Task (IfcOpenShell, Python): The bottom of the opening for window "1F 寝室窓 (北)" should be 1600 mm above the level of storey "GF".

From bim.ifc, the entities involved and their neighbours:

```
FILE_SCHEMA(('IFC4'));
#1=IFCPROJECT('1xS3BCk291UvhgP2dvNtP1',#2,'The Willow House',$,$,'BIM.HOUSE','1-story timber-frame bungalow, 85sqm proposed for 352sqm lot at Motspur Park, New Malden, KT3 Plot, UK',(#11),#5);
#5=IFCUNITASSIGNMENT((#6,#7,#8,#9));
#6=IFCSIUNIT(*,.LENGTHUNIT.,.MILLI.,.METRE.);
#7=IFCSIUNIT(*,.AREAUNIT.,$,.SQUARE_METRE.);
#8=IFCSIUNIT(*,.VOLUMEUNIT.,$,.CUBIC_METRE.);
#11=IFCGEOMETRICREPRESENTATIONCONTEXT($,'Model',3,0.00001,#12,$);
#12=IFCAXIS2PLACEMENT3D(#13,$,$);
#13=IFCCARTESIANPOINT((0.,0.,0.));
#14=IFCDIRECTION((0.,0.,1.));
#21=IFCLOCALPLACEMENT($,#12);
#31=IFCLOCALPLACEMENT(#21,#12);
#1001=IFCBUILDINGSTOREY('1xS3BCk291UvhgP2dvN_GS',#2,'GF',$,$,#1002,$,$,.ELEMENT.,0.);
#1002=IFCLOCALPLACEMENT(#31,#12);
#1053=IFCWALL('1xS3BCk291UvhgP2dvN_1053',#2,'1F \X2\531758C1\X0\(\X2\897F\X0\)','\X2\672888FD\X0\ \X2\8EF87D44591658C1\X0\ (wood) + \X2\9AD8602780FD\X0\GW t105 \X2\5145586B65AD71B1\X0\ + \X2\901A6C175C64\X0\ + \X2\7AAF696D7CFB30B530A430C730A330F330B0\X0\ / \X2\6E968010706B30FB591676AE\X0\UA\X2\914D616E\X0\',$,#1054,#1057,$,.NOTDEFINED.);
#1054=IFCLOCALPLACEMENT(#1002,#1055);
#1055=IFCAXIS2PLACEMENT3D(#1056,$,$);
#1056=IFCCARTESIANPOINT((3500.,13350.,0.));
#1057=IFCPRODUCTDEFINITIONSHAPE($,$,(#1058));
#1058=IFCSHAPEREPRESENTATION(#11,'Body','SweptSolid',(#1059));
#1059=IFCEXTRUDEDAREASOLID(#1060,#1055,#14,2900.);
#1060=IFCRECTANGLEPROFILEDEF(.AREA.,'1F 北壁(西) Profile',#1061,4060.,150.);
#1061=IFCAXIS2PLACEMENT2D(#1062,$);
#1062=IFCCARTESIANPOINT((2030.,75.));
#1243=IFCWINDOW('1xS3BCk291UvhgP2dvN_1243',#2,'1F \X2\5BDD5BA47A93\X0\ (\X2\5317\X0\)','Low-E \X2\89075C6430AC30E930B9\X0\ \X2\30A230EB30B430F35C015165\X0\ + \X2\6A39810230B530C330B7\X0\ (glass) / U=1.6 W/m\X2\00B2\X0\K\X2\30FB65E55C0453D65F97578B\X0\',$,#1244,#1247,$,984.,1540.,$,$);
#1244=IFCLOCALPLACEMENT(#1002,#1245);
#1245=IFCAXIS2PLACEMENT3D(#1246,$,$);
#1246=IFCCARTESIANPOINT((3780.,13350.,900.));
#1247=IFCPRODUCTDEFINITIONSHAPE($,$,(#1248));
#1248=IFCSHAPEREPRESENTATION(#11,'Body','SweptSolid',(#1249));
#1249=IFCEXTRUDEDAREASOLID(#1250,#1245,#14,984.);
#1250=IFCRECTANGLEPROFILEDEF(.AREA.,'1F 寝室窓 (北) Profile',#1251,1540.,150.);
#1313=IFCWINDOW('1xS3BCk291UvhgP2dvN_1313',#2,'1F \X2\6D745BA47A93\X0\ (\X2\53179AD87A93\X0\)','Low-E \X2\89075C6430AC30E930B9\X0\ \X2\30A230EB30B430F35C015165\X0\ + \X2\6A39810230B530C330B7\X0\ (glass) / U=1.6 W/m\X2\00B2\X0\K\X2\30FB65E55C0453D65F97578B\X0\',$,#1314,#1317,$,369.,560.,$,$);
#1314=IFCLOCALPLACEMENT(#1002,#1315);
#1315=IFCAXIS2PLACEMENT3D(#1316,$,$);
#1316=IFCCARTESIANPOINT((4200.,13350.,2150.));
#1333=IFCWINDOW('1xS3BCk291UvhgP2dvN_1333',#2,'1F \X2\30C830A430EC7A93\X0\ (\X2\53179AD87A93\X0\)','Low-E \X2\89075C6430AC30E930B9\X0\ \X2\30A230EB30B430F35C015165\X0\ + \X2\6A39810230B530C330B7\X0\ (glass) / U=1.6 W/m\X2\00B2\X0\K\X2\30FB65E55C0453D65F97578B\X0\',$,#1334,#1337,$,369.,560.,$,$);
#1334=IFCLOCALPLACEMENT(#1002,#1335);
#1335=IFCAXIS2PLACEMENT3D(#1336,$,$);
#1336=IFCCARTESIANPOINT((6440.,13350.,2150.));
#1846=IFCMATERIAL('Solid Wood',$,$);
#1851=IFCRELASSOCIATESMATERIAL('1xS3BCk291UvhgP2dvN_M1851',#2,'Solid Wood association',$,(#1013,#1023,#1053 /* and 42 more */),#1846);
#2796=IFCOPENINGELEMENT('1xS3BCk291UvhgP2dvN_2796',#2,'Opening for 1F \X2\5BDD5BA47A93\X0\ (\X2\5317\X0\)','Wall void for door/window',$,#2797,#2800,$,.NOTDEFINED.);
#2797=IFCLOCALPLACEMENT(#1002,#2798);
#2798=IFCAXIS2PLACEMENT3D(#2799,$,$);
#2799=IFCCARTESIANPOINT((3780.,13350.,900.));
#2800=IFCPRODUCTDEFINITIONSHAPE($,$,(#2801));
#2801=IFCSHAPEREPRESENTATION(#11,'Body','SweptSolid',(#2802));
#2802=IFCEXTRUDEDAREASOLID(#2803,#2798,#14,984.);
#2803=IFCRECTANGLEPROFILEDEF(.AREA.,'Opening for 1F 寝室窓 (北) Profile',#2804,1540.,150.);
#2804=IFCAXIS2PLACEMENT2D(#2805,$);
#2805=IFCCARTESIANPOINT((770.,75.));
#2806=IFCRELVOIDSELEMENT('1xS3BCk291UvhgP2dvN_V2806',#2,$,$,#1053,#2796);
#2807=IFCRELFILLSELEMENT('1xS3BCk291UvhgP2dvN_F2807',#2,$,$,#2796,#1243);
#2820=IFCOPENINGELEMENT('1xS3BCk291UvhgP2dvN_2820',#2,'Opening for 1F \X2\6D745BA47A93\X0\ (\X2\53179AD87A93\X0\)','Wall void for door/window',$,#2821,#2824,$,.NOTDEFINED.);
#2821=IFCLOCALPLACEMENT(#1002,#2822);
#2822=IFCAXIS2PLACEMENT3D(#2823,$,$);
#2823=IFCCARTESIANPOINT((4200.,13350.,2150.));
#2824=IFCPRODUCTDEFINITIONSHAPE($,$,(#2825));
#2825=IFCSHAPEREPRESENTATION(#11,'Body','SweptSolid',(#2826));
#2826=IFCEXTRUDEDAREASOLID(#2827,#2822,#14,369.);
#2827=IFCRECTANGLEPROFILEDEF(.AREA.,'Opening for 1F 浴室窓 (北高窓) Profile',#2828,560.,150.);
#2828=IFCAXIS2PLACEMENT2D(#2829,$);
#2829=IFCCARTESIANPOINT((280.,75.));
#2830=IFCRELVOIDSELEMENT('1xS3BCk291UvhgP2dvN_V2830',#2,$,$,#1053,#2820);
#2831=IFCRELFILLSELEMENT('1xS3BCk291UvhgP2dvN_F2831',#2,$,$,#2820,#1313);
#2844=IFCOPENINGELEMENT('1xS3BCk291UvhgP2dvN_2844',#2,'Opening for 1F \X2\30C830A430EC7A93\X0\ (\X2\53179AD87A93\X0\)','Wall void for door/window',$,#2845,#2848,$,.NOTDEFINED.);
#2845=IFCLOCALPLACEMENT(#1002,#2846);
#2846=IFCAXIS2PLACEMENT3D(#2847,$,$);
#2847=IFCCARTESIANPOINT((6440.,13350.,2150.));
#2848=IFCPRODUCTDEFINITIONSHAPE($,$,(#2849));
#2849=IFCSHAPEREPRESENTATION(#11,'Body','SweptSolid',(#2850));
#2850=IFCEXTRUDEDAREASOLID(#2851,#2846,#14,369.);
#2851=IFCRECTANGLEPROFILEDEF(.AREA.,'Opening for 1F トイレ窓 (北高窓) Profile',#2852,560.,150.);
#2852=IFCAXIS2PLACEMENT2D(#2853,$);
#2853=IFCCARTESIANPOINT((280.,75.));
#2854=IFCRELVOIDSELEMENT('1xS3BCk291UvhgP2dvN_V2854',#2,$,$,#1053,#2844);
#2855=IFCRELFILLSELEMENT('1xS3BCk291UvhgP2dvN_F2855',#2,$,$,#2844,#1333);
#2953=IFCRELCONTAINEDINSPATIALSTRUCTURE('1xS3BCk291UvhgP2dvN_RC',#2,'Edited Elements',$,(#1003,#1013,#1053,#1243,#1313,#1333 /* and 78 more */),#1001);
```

```python
import numpy as np
import ifcopenshell
import ifcopenshell.api.geometry
import ifcopenshell.geom
import ifcopenshell.util.element
import ifcopenshell.util.placement
import ifcopenshell.util.shape
import ifcopenshell.util.unit

model = ifcopenshell.open("bim.ifc")
unit_scale = ifcopenshell.util.unit.calculate_unit_scale(model)

window = model.by_guid("1xS3BCk291UvhgP2dvN_1243")
opening = window.FillsVoids[0].RelatingOpeningElement
storey = ifcopenshell.util.element.get_container(window, ifc_class="IfcBuildingStorey")
level = ifcopenshell.util.placement.get_local_placement(storey.ObjectPlacement)[2, 3]

# The opening's origin need not be at the sill, so measure its lowest point.
shape = ifcopenshell.geom.create_shape(ifcopenshell.geom.settings(), opening)
bottom = ifcopenshell.util.shape.get_shape_bottom_elevation(shape, shape.geometry) / unit_scale
dz = level + 1600.0 - bottom

shift = np.array([0.0, 0.0, dz])
# The window is not placed relative to its opening, so move both.
for product in (opening, window):
    matrix = ifcopenshell.util.placement.get_local_placement(product.ObjectPlacement)
    matrix[:3, 3] += shift
    ifcopenshell.api.geometry.edit_object_placement(model, product=product, matrix=matrix, is_si=False)

print(f"moved by {dz * unit_scale:+.3f} m")

model.write("bim_v2.ifc")
```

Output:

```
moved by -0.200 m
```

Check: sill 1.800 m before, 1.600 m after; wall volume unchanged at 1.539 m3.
